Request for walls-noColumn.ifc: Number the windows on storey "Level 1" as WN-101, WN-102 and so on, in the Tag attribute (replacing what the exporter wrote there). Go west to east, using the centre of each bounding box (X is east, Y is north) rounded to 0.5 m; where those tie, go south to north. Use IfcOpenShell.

First a look at what the model holds.

```python
import ifcopenshell
import ifcopenshell.util.element
import ifcopenshell.util.placement

model = ifcopenshell.open("walls-noColumn.ifc")
print(model.schema)
storey = next(s for s in model.by_type("IfcBuildingStorey") if s.Name == "Level 1")
windows = [e for e in ifcopenshell.util.element.get_decomposition(storey) if e.is_a("IfcWindow")]
for e in sorted(windows, key=lambda e: e.id()):
    origin = ifcopenshell.util.placement.get_local_placement(e.ObjectPlacement)[:3, 3]
    print(e.id(), e.Tag, e.Name, origin.round(2) + 0.0, sep=" | ")
```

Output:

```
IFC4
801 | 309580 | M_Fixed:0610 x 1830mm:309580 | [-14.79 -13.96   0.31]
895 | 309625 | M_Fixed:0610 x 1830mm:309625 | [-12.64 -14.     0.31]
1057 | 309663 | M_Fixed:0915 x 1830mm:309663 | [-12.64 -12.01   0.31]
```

```python
import ifcopenshell
import ifcopenshell.geom
import ifcopenshell.util.element
import ifcopenshell.util.shape

model = ifcopenshell.open("walls-noColumn.ifc")
settings = ifcopenshell.geom.settings()
settings.set("use-world-coords", True)


def centre(element):
    shape = ifcopenshell.geom.create_shape(settings, element)
    return ifcopenshell.util.shape.get_bbox_centroid(shape.geometry)


storey = next(s for s in model.by_type("IfcBuildingStorey") if s.Name == "Level 1")
windows = [e for e in ifcopenshell.util.element.get_decomposition(storey) if e.is_a("IfcWindow")]

# Insertion points can sit at a corner or the storey origin, so sort by the geometry (in metres).
centres = {e: centre(e) for e in windows}
windows.sort(key=lambda e: (round(centres[e][0] / 0.5), centres[e][1]))

for i, e in enumerate(windows, start=1):
    number = f"WN-1{i:02d}"
    e.Tag = number
    print(e.id(), number)

model.write("walls-noColumn_v2.ifc")
```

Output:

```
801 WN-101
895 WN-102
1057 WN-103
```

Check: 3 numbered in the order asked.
